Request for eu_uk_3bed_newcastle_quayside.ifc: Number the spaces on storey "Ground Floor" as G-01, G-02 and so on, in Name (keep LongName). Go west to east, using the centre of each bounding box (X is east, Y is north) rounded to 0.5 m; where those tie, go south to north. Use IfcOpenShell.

First a look at what the model holds.

```python
import ifcopenshell
import ifcopenshell.util.element
import ifcopenshell.util.placement

model = ifcopenshell.open("eu_uk_3bed_newcastle_quayside.ifc")
print(model.schema)
storey = next(s for s in model.by_type("IfcBuildingStorey") if s.Name == "Ground Floor")
spaces = [e for e in ifcopenshell.util.element.get_decomposition(storey) if e.is_a("IfcSpace")]
for e in sorted(spaces, key=lambda e: e.id()):
    origin = ifcopenshell.util.placement.get_local_placement(e.ObjectPlacement)[:3, 3]
    print(e.id(), e.Name, e.LongName, origin.round(2) + 0.0, sep=" | ")
```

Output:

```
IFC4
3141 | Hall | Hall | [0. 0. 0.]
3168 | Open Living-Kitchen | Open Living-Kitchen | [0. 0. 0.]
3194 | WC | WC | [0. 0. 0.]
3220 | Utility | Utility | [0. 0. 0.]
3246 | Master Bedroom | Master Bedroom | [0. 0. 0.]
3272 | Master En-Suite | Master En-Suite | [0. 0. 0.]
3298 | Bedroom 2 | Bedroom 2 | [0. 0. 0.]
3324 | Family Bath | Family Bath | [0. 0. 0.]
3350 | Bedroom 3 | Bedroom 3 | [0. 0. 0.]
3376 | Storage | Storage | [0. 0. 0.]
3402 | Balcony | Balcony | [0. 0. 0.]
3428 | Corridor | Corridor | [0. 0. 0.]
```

```python
import ifcopenshell
import ifcopenshell.geom
import ifcopenshell.util.element
import ifcopenshell.util.shape

model = ifcopenshell.open("eu_uk_3bed_newcastle_quayside.ifc")
settings = ifcopenshell.geom.settings()
settings.set("use-world-coords", True)


def centre(element):
    shape = ifcopenshell.geom.create_shape(settings, element)
    return ifcopenshell.util.shape.get_bbox_centroid(shape.geometry)


storey = next(s for s in model.by_type("IfcBuildingStorey") if s.Name == "Ground Floor")
spaces = [e for e in ifcopenshell.util.element.get_decomposition(storey) if e.is_a("IfcSpace")]

# Insertion points can sit at a corner or the storey origin, so sort by the geometry (in metres).
centres = {e: centre(e) for e in spaces}
spaces.sort(key=lambda e: (round(centres[e][0] / 0.5), centres[e][1]))

for i, e in enumerate(spaces, start=1):
    number = f"G-{i:02d}"
    e.Name = number
    print(e.id(), number)

model.write("eu_uk_3bed_newcastle_quayside_v2.ifc")
```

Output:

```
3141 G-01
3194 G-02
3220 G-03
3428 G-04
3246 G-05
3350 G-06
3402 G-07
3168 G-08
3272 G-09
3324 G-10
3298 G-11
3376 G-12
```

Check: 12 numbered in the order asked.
